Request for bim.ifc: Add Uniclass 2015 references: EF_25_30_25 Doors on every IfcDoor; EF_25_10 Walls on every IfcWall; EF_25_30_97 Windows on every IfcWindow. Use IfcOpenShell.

First a look at what the model holds.

```python
import ifcopenshell

model = ifcopenshell.open("bim.ifc")
print(model.schema)
print("classifications:", [c.Name for c in model.by_type("IfcClassification")])
for ifc_class in ("IfcDoor", "IfcRoof", "IfcStair", "IfcWall", "IfcWindow"):
    print(ifc_class, len(model.by_type(ifc_class)))
```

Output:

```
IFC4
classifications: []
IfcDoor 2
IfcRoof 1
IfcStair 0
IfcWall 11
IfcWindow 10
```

```python
import ifcopenshell
import ifcopenshell.api.classification

model = ifcopenshell.open("bim.ifc")

system = ifcopenshell.api.classification.add_classification(model, classification="Uniclass 2015")

codes = {
    "IfcDoor": ("EF_25_30_25", "Doors"),
    "IfcWall": ("EF_25_10", "Walls"),
    "IfcWindow": ("EF_25_30_97", "Windows"),
}
for ifc_class, (code, name) in codes.items():
    products = model.by_type(ifc_class)
    ifcopenshell.api.classification.add_reference(
        model, products=products, classification=system, identification=code, name=name
    )
    print(code, len(products))

model.write("bim_updated.ifc")
```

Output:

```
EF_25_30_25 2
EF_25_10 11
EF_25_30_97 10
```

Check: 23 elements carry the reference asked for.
